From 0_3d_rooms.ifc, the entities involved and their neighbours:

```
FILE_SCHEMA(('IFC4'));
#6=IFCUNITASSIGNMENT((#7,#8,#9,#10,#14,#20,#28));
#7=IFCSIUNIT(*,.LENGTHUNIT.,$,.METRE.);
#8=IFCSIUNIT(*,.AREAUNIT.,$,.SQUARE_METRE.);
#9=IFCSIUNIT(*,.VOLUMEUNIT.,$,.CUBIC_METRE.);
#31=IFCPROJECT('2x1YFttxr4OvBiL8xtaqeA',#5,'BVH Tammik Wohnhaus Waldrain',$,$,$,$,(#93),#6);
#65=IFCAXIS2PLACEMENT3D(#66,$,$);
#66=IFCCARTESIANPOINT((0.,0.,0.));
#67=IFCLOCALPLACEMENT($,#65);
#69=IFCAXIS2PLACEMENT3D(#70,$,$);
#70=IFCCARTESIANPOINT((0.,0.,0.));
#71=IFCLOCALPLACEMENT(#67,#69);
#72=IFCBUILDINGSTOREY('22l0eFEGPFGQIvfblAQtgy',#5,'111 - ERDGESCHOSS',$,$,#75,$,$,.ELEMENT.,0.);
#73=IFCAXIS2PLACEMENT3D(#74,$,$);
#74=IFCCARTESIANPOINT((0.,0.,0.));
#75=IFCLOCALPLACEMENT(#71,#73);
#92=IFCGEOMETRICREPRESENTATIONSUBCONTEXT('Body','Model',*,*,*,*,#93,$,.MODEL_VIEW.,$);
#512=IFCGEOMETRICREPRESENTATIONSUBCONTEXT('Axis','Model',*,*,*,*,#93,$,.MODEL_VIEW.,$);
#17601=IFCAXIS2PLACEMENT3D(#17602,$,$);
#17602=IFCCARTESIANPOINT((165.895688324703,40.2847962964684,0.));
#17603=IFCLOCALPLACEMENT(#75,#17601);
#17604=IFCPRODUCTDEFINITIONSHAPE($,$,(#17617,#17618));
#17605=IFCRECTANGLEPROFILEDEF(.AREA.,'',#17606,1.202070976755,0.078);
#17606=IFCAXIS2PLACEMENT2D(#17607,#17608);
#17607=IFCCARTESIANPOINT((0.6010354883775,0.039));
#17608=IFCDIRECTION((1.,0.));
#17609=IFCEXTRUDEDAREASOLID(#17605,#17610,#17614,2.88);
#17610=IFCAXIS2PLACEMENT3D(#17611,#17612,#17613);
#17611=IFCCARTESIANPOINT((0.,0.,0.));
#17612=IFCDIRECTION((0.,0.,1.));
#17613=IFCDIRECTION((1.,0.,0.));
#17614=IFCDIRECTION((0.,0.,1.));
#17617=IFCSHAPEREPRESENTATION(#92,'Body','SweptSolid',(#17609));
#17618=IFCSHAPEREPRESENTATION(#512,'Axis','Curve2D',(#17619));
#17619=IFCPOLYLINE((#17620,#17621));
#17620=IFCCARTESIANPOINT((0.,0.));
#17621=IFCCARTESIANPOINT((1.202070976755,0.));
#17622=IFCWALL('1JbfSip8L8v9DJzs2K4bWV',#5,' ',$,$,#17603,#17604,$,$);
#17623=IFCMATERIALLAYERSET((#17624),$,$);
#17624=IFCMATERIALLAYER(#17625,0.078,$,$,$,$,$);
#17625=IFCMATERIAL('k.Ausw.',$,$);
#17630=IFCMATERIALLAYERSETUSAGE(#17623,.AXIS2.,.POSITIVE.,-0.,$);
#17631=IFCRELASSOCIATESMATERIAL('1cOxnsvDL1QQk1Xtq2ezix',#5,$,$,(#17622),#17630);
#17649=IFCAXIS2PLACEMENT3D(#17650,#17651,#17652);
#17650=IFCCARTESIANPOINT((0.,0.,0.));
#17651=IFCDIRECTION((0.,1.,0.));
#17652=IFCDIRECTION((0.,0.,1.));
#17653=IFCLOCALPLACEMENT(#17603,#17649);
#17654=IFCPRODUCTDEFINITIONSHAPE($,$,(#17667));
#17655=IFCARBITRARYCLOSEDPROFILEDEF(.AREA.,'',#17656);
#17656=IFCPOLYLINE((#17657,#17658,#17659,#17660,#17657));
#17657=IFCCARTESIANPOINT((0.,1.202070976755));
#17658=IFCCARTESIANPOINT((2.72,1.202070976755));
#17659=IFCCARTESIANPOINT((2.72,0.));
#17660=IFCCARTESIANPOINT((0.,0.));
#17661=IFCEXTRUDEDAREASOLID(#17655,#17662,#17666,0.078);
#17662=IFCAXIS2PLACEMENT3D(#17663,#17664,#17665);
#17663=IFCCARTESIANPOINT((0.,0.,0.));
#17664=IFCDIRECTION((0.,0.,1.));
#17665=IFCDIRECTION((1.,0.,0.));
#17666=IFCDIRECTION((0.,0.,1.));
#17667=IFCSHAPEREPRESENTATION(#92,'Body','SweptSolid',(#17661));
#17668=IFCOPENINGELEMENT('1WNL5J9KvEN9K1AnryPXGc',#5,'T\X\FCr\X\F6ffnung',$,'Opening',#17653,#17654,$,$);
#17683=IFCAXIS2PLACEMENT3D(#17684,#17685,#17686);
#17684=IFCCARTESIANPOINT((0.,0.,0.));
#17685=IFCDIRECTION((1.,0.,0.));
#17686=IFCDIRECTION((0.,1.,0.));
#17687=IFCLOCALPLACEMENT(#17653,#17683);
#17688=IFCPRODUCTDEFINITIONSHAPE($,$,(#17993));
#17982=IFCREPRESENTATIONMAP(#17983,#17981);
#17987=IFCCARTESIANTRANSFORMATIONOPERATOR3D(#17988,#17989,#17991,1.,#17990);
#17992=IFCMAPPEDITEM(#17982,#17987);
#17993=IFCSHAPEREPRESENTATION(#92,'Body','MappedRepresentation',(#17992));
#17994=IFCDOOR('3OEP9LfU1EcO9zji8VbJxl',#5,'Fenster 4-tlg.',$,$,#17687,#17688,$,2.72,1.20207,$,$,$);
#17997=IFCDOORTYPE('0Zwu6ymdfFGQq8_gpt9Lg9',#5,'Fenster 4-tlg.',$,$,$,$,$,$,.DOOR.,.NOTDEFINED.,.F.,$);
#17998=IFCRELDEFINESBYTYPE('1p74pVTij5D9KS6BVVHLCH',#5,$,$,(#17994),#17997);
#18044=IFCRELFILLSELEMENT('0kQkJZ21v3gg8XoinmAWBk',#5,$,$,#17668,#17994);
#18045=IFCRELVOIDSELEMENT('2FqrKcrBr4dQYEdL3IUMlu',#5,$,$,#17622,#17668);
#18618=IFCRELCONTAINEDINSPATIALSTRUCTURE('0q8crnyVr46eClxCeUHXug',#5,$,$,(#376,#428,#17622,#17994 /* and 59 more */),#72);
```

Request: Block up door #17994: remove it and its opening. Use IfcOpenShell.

```python
import ifcopenshell
import ifcopenshell.api.feature
import ifcopenshell.api.root
import ifcopenshell.geom
import ifcopenshell.util.shape

model = ifcopenshell.open("0_3d_rooms.ifc")
settings = ifcopenshell.geom.settings()


def volume(element):
    """Net volume in cubic metres, openings subtracted."""
    shape = ifcopenshell.geom.create_shape(settings, element)
    return ifcopenshell.util.shape.get_volume(shape.geometry)


door = model.by_id(17994)
opening = door.FillsVoids[0].RelatingOpeningElement
wall = opening.VoidsElements[0].RelatingBuildingElement
before = volume(wall)

ifcopenshell.api.root.remove_product(model, product=door)
ifcopenshell.api.feature.remove_feature(model, feature=opening)

after = volume(wall)

print(f"wall volume {before:.3f} -> {after:.3f} m3")

model.write("0_3d_rooms_updated.ifc")
```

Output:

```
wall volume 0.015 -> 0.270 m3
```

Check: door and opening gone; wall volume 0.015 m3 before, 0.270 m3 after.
